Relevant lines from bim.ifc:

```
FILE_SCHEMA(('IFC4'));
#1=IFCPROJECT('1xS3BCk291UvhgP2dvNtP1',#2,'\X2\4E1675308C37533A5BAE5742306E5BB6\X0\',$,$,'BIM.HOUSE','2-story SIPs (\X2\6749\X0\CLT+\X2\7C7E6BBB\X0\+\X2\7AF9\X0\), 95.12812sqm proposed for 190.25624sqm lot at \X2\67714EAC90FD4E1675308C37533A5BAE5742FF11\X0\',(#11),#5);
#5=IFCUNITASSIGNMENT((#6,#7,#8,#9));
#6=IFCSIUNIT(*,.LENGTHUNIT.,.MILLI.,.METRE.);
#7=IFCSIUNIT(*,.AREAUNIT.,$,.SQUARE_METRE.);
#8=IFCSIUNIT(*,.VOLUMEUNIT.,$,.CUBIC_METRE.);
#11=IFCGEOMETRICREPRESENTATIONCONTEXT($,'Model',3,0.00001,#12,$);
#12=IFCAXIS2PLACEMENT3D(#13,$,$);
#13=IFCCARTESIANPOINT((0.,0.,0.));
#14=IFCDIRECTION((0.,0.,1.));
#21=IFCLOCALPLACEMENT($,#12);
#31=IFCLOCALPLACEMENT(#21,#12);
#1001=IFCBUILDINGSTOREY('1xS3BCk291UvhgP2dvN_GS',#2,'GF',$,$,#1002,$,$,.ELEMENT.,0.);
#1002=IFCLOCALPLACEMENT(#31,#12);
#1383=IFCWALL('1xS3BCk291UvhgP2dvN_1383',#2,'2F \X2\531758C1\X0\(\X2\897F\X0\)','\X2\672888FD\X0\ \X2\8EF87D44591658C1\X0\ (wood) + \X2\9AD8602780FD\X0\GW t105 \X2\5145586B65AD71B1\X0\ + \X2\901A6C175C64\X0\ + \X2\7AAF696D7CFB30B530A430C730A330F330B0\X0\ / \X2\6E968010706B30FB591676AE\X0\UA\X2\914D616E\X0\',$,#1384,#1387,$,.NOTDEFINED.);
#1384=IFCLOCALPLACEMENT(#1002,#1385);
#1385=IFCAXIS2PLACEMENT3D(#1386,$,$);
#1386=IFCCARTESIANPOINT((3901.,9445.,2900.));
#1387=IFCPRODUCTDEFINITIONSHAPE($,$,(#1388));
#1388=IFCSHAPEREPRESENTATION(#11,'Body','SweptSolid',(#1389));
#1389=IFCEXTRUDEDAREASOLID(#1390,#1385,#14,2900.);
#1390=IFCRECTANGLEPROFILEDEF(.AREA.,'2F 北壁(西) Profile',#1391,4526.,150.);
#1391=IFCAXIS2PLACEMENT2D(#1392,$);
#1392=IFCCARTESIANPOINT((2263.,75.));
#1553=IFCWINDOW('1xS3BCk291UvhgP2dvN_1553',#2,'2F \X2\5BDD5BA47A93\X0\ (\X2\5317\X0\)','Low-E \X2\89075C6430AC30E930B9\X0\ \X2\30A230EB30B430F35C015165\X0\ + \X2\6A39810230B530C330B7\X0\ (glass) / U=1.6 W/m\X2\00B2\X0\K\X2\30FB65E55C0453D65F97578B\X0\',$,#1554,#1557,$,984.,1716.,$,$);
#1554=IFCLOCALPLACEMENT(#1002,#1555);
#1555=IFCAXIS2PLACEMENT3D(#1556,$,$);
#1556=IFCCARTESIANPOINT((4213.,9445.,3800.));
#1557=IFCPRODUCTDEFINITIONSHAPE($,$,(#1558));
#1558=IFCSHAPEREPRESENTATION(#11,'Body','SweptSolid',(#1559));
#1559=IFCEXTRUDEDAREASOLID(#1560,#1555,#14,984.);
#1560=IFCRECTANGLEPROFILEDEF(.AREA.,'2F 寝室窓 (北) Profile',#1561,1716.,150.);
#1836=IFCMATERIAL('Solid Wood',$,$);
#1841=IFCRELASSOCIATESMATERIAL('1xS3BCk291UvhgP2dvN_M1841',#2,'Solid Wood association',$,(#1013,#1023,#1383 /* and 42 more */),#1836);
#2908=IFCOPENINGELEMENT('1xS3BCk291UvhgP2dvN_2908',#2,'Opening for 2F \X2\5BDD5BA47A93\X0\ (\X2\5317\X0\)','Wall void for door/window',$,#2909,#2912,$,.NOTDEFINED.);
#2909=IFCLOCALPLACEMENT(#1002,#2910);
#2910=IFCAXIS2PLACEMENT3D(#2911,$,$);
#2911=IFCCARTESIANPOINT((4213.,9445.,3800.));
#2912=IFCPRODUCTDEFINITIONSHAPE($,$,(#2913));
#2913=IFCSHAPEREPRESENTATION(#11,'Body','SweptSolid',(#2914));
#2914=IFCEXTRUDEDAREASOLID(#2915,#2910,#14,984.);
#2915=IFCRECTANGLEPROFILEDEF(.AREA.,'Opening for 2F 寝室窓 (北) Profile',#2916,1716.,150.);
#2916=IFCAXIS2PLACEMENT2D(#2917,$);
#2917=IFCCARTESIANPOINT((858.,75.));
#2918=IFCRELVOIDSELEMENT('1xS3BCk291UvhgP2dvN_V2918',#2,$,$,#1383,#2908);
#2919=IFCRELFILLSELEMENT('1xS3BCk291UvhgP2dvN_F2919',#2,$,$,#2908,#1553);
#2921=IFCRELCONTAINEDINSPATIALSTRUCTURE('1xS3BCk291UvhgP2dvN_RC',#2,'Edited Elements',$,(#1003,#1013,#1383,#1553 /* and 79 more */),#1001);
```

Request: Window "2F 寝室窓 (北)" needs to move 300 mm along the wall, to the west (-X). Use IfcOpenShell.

```python
import ifcopenshell
import ifcopenshell.api.geometry
import ifcopenshell.util.placement
import ifcopenshell.util.unit

model = ifcopenshell.open("bim.ifc")
unit_scale = ifcopenshell.util.unit.calculate_unit_scale(model)

window = model.by_guid("1xS3BCk291UvhgP2dvN_1553")
opening = window.FillsVoids[0].RelatingOpeningElement
wall = opening.VoidsElements[0].RelatingBuildingElement

wall_matrix = ifcopenshell.util.placement.get_local_placement(wall.ObjectPlacement)
shift = wall_matrix[:3, 0] * -0.3 / unit_scale
before = ifcopenshell.util.placement.get_local_placement(window.ObjectPlacement)[:3, 3].copy()

# The window is not placed relative to its opening, so move both.
for product in (opening, window):
    matrix = ifcopenshell.util.placement.get_local_placement(product.ObjectPlacement)
    matrix[:3, 3] += shift
    ifcopenshell.api.geometry.edit_object_placement(model, product=product, matrix=matrix, is_si=False)

after = ifcopenshell.util.placement.get_local_placement(window.ObjectPlacement)[:3, 3]
print("window moved by", (after - before).round(3) + 0.0)

model.write("bim-out.ifc")
```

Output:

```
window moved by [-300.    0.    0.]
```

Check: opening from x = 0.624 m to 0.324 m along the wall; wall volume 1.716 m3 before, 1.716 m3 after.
